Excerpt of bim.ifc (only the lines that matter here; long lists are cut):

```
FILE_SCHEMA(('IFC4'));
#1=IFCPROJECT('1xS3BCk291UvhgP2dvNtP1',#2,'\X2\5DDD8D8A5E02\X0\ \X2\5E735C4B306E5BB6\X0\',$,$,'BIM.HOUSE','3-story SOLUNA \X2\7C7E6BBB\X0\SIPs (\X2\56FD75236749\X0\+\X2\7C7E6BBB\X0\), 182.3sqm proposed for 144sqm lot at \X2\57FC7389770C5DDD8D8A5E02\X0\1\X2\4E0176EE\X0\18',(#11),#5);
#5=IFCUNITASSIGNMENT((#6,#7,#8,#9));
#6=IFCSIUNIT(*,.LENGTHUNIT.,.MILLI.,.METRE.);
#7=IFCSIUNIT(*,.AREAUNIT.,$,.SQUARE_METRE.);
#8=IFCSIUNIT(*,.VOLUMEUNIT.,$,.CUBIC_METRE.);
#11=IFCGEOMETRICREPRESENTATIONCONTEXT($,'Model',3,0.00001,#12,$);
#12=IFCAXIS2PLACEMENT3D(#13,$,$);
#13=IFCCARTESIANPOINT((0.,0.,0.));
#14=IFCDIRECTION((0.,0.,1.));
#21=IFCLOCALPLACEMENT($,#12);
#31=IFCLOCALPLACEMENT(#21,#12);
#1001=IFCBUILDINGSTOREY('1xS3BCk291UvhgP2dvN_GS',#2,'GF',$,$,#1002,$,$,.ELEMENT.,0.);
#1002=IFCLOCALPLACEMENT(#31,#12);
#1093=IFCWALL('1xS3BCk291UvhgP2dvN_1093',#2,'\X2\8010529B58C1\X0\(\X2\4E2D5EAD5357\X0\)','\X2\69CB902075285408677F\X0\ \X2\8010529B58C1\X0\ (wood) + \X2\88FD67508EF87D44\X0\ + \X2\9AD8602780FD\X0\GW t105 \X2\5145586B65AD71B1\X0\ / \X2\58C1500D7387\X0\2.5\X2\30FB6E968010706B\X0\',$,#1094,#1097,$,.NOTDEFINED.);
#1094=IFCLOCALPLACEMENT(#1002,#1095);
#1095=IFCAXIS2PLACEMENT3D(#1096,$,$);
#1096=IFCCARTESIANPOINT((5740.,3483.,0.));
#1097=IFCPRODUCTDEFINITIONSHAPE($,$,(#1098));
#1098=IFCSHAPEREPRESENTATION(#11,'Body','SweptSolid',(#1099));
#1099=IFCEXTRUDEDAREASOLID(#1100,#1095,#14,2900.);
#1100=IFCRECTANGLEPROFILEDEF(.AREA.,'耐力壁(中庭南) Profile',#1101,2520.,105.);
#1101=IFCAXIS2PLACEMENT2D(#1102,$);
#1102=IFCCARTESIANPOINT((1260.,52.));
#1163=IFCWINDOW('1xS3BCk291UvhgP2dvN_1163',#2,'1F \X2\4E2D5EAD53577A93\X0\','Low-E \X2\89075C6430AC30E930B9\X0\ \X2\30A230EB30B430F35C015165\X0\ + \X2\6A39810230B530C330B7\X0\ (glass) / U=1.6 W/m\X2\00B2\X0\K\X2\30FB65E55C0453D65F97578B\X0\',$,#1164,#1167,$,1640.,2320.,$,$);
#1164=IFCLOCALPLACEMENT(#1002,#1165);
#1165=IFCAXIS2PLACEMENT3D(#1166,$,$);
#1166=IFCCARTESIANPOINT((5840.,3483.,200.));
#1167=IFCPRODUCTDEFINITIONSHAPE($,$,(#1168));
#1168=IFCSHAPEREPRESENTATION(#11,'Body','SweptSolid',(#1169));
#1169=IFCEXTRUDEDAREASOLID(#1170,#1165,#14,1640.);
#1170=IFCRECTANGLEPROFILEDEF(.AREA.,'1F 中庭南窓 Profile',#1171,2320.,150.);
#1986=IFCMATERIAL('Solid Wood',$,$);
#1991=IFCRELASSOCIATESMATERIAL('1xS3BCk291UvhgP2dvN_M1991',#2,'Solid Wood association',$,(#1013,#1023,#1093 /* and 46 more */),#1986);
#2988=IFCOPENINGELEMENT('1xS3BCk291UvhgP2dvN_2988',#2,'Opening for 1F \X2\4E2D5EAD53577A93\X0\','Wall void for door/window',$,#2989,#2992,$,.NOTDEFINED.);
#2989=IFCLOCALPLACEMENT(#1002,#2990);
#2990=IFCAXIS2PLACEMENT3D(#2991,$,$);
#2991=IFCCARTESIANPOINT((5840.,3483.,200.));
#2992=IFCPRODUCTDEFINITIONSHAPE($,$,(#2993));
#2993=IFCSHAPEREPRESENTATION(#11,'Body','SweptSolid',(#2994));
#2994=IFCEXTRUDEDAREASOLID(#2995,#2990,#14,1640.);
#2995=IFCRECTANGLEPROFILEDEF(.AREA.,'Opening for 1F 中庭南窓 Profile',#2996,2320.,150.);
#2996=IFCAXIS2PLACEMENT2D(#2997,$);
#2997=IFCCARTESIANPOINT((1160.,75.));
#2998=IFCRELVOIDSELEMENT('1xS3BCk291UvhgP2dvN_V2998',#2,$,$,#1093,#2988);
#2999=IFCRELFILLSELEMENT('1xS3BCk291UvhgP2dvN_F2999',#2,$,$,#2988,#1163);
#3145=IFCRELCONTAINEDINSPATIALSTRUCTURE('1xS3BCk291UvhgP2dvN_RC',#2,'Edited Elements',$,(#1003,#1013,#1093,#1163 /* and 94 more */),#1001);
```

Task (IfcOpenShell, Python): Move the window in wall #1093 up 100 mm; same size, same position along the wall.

```python
import numpy as np
import ifcopenshell
import ifcopenshell.api.geometry
import ifcopenshell.util.placement
import ifcopenshell.util.unit

model = ifcopenshell.open("bim.ifc")
unit_scale = ifcopenshell.util.unit.calculate_unit_scale(model)

window = model.by_guid("1xS3BCk291UvhgP2dvN_1163")
opening = window.FillsVoids[0].RelatingOpeningElement
dz = 0.1 / unit_scale

shift = np.array([0.0, 0.0, dz])
# The window is not placed relative to its opening, so move both.
for product in (opening, window):
    matrix = ifcopenshell.util.placement.get_local_placement(product.ObjectPlacement)
    matrix[:3, 3] += shift
    ifcopenshell.api.geometry.edit_object_placement(model, product=product, matrix=matrix, is_si=False)

print(f"moved by {dz * unit_scale:+.3f} m")

model.write("bim_rev.ifc")
```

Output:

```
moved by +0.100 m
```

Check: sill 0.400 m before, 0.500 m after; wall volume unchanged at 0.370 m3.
